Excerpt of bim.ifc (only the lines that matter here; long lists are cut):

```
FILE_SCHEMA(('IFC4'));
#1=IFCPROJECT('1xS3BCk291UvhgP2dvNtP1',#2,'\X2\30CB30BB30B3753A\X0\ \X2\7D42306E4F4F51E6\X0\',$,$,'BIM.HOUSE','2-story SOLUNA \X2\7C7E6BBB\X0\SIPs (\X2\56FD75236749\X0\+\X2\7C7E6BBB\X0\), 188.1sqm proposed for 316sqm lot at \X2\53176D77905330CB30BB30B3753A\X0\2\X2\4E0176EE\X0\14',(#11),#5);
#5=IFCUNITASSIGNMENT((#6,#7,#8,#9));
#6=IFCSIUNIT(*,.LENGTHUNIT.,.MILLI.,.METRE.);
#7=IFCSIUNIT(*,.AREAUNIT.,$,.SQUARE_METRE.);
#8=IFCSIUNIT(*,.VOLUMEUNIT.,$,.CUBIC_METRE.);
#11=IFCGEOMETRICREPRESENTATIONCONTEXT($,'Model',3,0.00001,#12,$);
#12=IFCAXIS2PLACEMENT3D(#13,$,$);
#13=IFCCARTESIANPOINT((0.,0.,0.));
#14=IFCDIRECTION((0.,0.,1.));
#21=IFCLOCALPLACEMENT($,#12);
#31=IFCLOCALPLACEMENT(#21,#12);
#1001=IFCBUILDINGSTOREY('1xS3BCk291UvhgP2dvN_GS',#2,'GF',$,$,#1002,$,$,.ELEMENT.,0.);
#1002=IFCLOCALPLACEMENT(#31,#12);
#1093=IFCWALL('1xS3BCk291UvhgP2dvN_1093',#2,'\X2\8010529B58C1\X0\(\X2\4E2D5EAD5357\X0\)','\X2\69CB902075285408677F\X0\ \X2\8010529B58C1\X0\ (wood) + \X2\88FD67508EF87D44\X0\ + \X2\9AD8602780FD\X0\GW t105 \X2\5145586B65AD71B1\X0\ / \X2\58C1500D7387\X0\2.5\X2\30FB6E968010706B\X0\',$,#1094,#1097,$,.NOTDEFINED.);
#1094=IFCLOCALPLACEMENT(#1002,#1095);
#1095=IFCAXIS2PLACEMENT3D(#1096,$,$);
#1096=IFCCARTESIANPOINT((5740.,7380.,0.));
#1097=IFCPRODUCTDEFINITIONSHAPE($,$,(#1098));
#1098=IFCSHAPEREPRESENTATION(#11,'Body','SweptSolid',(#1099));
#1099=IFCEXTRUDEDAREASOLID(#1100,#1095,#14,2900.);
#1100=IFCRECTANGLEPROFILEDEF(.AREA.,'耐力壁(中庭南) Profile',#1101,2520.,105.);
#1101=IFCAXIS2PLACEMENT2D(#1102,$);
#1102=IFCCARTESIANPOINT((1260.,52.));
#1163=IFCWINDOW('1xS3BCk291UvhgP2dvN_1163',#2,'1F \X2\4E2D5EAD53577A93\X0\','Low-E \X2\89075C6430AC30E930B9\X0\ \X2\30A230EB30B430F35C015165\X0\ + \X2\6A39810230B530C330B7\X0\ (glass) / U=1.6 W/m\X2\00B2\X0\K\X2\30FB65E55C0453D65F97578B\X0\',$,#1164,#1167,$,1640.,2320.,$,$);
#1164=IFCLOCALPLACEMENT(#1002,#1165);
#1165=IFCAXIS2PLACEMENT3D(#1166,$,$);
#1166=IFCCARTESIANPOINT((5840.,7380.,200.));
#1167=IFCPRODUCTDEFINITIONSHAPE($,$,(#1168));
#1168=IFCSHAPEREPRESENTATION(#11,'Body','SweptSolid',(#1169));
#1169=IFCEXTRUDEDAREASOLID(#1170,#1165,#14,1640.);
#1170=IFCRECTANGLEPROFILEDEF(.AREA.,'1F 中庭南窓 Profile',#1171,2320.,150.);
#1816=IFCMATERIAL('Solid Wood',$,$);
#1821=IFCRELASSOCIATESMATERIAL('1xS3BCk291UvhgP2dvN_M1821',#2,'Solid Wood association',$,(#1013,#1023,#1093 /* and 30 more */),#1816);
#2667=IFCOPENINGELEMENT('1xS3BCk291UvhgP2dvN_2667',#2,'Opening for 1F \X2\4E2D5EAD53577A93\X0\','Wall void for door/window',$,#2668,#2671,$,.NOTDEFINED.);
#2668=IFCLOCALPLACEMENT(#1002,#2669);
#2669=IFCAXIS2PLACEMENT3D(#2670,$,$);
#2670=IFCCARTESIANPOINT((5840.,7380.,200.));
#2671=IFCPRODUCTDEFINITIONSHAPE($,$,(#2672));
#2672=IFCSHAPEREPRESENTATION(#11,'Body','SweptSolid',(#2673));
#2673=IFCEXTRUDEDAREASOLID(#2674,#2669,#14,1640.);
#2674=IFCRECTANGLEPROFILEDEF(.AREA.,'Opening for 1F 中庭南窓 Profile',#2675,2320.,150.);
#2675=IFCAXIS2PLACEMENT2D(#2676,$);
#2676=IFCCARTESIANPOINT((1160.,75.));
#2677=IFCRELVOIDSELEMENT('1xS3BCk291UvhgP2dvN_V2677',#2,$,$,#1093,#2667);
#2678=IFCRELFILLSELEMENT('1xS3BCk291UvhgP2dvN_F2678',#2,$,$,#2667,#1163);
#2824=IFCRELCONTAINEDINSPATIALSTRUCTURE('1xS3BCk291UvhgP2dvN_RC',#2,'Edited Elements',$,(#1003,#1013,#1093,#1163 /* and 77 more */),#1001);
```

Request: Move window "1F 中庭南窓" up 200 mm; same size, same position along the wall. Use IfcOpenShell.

```python
import numpy as np
import ifcopenshell
import ifcopenshell.api.geometry
import ifcopenshell.util.placement
import ifcopenshell.util.unit

model = ifcopenshell.open("bim.ifc")
unit_scale = ifcopenshell.util.unit.calculate_unit_scale(model)

window = model.by_guid("1xS3BCk291UvhgP2dvN_1163")
opening = window.FillsVoids[0].RelatingOpeningElement
dz = 0.2 / unit_scale

shift = np.array([0.0, 0.0, dz])
# The window is not placed relative to its opening, so move both.
for product in (opening, window):
    matrix = ifcopenshell.util.placement.get_local_placement(product.ObjectPlacement)
    matrix[:3, 3] += shift
    ifcopenshell.api.geometry.edit_object_placement(model, product=product, matrix=matrix, is_si=False)

print(f"moved by {dz * unit_scale:+.3f} m")

model.write("bim_updated.ifc")
```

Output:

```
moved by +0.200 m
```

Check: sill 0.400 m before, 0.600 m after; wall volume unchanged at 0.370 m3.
